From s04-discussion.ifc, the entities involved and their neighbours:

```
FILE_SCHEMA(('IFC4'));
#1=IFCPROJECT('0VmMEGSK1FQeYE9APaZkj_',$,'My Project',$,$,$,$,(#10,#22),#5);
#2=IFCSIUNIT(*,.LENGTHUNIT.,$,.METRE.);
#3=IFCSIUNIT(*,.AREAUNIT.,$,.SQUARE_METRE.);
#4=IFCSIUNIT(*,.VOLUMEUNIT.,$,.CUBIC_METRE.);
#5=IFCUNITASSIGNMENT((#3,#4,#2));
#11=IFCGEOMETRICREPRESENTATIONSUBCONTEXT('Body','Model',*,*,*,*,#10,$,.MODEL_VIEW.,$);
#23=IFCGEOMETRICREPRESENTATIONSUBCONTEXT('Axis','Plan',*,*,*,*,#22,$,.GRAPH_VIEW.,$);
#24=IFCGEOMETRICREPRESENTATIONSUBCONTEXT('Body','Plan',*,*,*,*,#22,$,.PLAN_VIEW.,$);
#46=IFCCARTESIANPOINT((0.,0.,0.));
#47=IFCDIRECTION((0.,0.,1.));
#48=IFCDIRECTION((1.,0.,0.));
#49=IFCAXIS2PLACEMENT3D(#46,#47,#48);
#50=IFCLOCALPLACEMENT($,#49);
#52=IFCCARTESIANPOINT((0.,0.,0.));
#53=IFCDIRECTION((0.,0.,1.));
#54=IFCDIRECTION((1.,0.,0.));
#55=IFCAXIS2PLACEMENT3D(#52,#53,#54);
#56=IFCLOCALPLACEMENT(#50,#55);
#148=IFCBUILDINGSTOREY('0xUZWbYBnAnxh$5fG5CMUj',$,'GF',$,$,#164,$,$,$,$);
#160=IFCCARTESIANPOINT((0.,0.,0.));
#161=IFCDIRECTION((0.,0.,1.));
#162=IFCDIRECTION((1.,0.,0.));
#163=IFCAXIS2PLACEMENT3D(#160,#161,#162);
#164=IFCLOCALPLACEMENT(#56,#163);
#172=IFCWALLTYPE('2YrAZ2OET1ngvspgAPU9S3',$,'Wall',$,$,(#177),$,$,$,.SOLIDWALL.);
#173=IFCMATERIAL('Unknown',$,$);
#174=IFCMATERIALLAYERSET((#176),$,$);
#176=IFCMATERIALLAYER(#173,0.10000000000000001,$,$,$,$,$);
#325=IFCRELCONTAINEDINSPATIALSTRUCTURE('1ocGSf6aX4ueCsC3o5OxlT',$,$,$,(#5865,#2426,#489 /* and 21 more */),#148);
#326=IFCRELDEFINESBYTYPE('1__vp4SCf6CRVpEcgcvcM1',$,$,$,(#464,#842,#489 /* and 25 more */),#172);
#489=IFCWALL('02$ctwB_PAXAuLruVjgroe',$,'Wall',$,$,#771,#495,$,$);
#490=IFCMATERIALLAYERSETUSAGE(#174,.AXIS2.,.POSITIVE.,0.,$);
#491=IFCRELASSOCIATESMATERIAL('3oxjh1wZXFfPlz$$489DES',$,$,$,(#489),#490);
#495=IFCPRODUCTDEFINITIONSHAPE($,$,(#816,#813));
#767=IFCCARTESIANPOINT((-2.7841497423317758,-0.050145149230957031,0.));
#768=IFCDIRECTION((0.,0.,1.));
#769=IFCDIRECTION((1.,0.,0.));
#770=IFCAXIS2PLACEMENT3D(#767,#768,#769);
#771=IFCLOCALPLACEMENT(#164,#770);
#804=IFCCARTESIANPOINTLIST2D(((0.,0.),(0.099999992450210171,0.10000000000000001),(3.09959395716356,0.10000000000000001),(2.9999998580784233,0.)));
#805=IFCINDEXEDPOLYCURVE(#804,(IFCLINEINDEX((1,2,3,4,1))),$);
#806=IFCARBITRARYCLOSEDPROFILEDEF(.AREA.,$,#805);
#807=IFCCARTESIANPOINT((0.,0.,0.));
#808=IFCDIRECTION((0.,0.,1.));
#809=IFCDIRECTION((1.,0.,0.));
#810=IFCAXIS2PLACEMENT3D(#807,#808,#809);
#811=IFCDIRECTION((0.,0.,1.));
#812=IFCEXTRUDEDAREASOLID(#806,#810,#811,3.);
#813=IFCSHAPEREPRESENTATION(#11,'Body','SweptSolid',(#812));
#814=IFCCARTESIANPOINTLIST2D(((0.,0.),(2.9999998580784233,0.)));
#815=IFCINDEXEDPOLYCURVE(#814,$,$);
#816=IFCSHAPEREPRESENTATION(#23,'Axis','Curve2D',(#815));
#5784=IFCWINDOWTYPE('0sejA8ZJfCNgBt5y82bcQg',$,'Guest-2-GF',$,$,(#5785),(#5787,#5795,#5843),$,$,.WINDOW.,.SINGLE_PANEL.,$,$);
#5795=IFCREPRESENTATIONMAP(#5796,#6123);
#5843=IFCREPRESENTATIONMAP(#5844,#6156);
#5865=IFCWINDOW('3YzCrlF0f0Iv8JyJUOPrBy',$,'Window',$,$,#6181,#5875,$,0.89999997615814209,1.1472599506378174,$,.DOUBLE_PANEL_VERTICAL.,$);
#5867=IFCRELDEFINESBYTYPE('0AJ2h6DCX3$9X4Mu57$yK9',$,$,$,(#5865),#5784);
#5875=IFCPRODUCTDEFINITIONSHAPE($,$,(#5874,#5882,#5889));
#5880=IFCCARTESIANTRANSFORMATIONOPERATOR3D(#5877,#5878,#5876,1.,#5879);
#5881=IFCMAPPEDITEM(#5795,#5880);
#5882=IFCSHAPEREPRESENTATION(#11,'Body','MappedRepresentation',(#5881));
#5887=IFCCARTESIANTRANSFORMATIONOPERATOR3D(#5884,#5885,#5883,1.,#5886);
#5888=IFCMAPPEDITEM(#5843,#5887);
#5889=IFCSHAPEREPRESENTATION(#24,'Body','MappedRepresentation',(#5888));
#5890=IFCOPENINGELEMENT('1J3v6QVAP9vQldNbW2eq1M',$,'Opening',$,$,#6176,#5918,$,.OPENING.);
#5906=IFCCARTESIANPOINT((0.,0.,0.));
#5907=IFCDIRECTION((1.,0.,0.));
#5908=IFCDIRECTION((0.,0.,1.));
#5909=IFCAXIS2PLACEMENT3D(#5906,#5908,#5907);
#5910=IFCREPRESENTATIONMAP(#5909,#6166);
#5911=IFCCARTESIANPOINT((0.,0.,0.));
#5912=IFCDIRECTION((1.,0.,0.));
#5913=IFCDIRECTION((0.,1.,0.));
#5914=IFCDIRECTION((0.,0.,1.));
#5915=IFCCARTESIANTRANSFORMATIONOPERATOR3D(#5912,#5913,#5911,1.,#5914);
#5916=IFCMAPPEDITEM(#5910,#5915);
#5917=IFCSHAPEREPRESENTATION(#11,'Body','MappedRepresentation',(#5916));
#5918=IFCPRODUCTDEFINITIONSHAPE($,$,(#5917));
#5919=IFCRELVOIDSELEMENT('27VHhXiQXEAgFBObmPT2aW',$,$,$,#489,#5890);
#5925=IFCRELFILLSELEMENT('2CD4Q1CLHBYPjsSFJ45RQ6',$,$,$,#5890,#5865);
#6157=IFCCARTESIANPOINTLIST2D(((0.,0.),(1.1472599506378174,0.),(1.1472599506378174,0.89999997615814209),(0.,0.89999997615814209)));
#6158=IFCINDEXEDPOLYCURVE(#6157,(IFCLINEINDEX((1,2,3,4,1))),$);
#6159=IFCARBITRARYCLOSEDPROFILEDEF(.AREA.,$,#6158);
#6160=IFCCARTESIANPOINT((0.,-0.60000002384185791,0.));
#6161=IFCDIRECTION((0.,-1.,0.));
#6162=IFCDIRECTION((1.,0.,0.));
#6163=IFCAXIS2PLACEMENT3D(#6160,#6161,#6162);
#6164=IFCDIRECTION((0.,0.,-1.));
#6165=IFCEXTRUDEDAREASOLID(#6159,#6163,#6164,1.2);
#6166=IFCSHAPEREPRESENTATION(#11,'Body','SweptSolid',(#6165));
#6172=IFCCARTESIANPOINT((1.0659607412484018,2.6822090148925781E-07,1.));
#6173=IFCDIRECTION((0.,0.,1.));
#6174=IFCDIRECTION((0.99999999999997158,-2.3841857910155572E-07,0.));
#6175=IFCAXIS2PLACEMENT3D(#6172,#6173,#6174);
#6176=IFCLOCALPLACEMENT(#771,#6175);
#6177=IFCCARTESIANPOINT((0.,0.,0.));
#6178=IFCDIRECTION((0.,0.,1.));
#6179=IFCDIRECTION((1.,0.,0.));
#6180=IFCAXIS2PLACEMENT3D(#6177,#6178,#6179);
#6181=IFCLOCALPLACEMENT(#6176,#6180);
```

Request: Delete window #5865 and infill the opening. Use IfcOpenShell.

```python
import ifcopenshell
import ifcopenshell.api.feature
import ifcopenshell.api.root
import ifcopenshell.geom
import ifcopenshell.util.shape

model = ifcopenshell.open("s04-discussion.ifc")
settings = ifcopenshell.geom.settings()


def volume(element):
    """Net volume in cubic metres, openings subtracted."""
    shape = ifcopenshell.geom.create_shape(settings, element)
    return ifcopenshell.util.shape.get_volume(shape.geometry)


window = model.by_id(5865)
opening = window.FillsVoids[0].RelatingOpeningElement
wall = opening.VoidsElements[0].RelatingBuildingElement
before = volume(wall)

ifcopenshell.api.root.remove_product(model, product=window)
ifcopenshell.api.feature.remove_feature(model, feature=opening)

after = volume(wall)

print(f"wall volume {before:.3f} -> {after:.3f} m3")

model.write("s04-discussion-out.ifc")
```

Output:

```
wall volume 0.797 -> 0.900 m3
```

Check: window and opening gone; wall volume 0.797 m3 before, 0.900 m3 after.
